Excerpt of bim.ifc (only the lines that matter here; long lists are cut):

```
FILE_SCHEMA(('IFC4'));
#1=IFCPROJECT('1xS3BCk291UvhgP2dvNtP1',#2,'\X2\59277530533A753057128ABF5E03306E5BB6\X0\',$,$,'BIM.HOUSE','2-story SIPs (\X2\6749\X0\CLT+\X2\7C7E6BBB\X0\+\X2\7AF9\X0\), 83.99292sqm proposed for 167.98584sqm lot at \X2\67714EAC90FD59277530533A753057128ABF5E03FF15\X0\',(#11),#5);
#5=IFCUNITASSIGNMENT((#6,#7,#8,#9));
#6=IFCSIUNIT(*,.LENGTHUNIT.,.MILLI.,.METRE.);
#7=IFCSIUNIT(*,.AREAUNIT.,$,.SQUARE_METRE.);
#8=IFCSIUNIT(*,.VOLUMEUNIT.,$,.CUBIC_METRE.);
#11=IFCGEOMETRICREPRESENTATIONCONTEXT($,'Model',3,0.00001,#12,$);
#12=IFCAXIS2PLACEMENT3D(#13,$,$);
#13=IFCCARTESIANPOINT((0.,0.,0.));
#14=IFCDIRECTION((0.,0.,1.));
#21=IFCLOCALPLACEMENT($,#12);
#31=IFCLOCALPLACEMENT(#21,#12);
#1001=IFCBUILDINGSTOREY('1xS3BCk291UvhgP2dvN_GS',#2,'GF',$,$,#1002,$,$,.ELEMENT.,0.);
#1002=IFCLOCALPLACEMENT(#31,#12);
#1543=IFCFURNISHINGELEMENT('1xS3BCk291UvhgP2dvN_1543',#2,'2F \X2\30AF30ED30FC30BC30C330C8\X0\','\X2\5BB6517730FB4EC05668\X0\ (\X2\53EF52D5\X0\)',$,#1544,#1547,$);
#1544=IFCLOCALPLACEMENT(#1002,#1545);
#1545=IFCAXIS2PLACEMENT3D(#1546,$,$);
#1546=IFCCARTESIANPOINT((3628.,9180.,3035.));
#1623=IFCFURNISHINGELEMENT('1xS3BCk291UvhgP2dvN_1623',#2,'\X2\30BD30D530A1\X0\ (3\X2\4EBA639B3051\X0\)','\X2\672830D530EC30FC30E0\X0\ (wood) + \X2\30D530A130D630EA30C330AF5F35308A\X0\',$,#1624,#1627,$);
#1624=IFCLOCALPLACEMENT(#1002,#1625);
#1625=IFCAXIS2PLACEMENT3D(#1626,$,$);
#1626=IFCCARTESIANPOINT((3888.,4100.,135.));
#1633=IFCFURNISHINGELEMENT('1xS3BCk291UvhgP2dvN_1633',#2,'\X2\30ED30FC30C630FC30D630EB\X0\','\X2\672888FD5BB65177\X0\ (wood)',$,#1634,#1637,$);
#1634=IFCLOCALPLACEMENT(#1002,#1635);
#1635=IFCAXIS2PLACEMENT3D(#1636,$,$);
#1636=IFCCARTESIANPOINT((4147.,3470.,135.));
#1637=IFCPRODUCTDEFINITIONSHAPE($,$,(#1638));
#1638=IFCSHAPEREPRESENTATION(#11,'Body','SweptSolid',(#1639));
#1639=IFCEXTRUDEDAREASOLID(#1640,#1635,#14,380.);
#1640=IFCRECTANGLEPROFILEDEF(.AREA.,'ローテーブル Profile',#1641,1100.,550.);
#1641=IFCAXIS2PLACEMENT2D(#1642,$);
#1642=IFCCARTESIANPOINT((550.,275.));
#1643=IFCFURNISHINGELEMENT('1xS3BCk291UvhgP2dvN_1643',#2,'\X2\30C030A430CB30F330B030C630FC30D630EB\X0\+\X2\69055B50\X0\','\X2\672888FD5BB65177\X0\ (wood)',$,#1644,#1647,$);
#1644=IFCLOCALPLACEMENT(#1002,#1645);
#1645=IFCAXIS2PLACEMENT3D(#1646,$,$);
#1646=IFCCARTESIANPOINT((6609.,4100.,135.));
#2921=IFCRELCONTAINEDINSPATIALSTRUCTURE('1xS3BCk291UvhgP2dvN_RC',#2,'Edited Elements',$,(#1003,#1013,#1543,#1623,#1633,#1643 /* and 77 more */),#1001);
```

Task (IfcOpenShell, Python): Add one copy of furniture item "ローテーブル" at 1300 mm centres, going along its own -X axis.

```python
import ifcopenshell
import ifcopenshell.api.geometry
import ifcopenshell.api.root
import ifcopenshell.util.element
import ifcopenshell.util.placement
import ifcopenshell.util.unit

model = ifcopenshell.open("bim.ifc")
unit_scale = ifcopenshell.util.unit.calculate_unit_scale(model)


def reuse_history(source, copy):
    """copy_class also copies each property set's owner history, people and application; keep the originals."""
    for rel in copy.IsDefinedBy:
        if rel.is_a("IfcRelDefinesByProperties") and (history := rel.RelatingPropertyDefinition.OwnerHistory):
            rel.RelatingPropertyDefinition.OwnerHistory = source.OwnerHistory
            ifcopenshell.util.element.remove_deep2(model, history)


source = model.by_id(1633)
base = ifcopenshell.util.placement.get_local_placement(source.ObjectPlacement)
step = -base[:3, 0] * 1.3 / unit_scale

for i in range(1, 2):
    copy = ifcopenshell.api.root.copy_class(model, product=source)
    copy.Representation = ifcopenshell.util.element.copy_deep(
        model, source.Representation, exclude=["IfcGeometricRepresentationContext", "IfcRepresentationMap"]
    )
    reuse_history(source, copy)
    matrix = base.copy()
    matrix[:3, 3] += i * step
    print("added at", matrix[:3, 3].round(3) + 0.0)
    ifcopenshell.api.geometry.edit_object_placement(model, product=copy, matrix=matrix, is_si=False)

model.write("bim_v2.ifc")
```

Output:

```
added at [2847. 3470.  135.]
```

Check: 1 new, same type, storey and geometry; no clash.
